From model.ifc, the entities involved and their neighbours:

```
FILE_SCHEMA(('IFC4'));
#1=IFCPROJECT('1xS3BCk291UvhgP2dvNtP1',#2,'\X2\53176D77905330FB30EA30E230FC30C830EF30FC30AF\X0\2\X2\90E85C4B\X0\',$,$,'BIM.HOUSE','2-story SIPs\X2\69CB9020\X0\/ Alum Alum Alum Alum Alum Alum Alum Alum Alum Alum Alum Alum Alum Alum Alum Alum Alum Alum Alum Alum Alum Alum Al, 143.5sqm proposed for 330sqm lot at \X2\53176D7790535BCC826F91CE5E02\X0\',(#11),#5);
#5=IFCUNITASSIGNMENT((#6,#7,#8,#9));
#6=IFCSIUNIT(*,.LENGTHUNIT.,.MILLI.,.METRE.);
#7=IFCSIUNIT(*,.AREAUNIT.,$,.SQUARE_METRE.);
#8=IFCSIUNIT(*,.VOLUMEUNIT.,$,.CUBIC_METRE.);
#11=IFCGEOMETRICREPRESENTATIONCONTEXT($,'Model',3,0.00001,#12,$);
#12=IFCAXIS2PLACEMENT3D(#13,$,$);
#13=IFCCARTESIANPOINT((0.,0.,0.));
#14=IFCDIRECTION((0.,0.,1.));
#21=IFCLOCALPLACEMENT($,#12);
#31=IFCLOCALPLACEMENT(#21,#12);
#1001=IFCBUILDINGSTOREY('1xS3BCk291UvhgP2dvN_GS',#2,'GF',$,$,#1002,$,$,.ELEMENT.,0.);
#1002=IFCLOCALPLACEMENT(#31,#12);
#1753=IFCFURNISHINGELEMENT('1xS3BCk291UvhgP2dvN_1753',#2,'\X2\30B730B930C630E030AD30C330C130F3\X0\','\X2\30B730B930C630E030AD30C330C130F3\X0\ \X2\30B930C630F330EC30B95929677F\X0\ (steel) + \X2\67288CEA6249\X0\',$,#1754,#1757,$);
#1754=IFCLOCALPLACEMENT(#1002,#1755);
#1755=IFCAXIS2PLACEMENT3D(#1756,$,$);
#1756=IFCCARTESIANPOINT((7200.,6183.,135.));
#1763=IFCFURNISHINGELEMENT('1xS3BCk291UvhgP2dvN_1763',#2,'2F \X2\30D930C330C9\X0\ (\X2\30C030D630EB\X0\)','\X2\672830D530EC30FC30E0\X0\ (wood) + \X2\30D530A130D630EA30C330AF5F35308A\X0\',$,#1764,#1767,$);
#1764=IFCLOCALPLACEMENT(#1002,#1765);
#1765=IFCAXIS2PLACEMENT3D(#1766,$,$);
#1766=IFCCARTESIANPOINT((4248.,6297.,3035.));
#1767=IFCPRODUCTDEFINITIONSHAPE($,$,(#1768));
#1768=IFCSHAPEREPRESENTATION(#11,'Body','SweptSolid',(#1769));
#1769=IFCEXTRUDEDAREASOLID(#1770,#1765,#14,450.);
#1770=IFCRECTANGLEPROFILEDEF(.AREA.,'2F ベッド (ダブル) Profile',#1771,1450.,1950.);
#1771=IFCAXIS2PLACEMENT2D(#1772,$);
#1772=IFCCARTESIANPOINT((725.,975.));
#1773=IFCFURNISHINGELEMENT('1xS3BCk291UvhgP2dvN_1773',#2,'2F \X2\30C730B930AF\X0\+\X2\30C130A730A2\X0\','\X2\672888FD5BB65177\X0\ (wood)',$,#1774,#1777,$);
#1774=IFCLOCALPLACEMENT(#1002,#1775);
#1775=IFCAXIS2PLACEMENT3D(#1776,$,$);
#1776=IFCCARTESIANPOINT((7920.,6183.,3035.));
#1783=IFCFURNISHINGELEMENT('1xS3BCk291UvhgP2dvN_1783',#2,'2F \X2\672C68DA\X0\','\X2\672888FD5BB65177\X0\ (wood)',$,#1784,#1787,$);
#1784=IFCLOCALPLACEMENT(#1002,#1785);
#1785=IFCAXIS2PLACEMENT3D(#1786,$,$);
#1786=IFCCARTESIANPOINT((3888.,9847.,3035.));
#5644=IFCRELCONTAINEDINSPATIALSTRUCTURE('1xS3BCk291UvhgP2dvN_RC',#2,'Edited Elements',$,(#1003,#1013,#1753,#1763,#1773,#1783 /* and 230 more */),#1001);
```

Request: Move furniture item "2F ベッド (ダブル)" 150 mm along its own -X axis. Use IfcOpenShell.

```python
import ifcopenshell
import ifcopenshell.api.geometry
import ifcopenshell.util.placement

model = ifcopenshell.open("model.ifc")

item = model.by_id(1763)
matrix = ifcopenshell.util.placement.get_local_placement(item.ObjectPlacement)
matrix[:3, 3] -= matrix[:3, 0] * 150.0
ifcopenshell.api.geometry.edit_object_placement(model, product=item, matrix=matrix, is_si=False)

print(ifcopenshell.util.placement.get_local_placement(item.ObjectPlacement).round(3) + 0.0)

model.write("model-out.ifc")
```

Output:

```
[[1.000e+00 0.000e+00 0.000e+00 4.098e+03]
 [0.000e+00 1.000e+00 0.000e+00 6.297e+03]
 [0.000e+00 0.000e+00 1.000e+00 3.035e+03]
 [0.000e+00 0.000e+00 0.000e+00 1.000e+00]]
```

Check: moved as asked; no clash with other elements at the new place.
